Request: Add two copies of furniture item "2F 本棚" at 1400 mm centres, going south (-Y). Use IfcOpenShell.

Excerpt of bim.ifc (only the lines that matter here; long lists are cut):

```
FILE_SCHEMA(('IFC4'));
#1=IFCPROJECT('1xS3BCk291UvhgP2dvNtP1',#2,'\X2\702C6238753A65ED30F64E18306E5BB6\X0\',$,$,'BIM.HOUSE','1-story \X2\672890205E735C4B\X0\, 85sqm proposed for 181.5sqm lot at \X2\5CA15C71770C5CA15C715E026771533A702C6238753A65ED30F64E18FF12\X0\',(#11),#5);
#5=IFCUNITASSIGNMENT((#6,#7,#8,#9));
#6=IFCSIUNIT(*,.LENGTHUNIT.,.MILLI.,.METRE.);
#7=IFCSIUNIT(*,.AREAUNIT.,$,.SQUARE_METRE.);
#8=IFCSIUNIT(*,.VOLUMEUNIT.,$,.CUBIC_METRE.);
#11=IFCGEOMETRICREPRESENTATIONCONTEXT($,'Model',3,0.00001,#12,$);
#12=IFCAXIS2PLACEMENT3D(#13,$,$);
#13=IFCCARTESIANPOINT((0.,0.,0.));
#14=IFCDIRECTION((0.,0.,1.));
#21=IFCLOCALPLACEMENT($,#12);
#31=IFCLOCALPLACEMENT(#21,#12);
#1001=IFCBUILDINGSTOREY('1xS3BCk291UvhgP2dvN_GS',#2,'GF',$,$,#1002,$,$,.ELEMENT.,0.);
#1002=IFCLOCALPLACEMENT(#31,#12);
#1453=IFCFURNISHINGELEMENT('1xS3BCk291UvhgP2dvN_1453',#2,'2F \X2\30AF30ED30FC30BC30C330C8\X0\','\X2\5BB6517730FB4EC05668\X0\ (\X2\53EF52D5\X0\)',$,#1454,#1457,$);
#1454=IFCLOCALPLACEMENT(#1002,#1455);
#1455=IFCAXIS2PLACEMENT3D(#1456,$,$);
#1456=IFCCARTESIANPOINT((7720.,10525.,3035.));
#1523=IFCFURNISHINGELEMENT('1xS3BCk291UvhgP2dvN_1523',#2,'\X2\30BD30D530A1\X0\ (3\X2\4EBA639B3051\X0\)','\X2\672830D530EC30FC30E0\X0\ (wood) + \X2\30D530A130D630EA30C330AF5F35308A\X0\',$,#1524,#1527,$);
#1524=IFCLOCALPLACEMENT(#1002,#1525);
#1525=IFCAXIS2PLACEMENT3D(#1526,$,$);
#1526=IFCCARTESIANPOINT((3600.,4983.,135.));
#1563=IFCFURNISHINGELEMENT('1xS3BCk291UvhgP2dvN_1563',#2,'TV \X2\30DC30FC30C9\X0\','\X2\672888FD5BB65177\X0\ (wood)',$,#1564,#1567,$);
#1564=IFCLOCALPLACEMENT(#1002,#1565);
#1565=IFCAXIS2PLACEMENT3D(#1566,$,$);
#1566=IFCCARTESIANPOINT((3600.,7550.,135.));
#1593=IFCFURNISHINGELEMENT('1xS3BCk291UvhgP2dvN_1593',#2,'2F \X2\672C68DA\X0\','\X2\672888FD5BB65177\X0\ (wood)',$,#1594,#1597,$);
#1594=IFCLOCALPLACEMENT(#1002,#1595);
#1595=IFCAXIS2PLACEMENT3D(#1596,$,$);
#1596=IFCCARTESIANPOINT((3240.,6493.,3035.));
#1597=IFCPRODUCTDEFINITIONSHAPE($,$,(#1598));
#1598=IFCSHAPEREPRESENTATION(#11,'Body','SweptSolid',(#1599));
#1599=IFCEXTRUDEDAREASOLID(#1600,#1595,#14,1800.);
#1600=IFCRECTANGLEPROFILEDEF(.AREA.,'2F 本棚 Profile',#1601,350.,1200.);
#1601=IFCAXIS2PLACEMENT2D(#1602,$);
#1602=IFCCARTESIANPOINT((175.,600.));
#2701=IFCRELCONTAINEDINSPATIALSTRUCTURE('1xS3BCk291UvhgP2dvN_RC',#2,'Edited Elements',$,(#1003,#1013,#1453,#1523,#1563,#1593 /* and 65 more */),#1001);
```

```python
import numpy as np
import ifcopenshell
import ifcopenshell.api.geometry
import ifcopenshell.api.root
import ifcopenshell.util.element
import ifcopenshell.util.placement
import ifcopenshell.util.unit

model = ifcopenshell.open("bim.ifc")
unit_scale = ifcopenshell.util.unit.calculate_unit_scale(model)


def reuse_history(source, copy):
    """copy_class also copies each property set's owner history, people and application; keep the originals."""
    for rel in copy.IsDefinedBy:
        if rel.is_a("IfcRelDefinesByProperties") and (history := rel.RelatingPropertyDefinition.OwnerHistory):
            rel.RelatingPropertyDefinition.OwnerHistory = source.OwnerHistory
            ifcopenshell.util.element.remove_deep2(model, history)


source = model.by_guid("1xS3BCk291UvhgP2dvN_1593")
base = ifcopenshell.util.placement.get_local_placement(source.ObjectPlacement)
step = np.array([0.0, -1.0, 0.0]) * 1.4 / unit_scale

for i in range(1, 3):
    copy = ifcopenshell.api.root.copy_class(model, product=source)
    copy.Representation = ifcopenshell.util.element.copy_deep(
        model, source.Representation, exclude=["IfcGeometricRepresentationContext", "IfcRepresentationMap"]
    )
    reuse_history(source, copy)
    matrix = base.copy()
    matrix[:3, 3] += i * step
    print("added at", matrix[:3, 3].round(3) + 0.0)
    ifcopenshell.api.geometry.edit_object_placement(model, product=copy, matrix=matrix, is_si=False)

model.write("bim-out.ifc")
```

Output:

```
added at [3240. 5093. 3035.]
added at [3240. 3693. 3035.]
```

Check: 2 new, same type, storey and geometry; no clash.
